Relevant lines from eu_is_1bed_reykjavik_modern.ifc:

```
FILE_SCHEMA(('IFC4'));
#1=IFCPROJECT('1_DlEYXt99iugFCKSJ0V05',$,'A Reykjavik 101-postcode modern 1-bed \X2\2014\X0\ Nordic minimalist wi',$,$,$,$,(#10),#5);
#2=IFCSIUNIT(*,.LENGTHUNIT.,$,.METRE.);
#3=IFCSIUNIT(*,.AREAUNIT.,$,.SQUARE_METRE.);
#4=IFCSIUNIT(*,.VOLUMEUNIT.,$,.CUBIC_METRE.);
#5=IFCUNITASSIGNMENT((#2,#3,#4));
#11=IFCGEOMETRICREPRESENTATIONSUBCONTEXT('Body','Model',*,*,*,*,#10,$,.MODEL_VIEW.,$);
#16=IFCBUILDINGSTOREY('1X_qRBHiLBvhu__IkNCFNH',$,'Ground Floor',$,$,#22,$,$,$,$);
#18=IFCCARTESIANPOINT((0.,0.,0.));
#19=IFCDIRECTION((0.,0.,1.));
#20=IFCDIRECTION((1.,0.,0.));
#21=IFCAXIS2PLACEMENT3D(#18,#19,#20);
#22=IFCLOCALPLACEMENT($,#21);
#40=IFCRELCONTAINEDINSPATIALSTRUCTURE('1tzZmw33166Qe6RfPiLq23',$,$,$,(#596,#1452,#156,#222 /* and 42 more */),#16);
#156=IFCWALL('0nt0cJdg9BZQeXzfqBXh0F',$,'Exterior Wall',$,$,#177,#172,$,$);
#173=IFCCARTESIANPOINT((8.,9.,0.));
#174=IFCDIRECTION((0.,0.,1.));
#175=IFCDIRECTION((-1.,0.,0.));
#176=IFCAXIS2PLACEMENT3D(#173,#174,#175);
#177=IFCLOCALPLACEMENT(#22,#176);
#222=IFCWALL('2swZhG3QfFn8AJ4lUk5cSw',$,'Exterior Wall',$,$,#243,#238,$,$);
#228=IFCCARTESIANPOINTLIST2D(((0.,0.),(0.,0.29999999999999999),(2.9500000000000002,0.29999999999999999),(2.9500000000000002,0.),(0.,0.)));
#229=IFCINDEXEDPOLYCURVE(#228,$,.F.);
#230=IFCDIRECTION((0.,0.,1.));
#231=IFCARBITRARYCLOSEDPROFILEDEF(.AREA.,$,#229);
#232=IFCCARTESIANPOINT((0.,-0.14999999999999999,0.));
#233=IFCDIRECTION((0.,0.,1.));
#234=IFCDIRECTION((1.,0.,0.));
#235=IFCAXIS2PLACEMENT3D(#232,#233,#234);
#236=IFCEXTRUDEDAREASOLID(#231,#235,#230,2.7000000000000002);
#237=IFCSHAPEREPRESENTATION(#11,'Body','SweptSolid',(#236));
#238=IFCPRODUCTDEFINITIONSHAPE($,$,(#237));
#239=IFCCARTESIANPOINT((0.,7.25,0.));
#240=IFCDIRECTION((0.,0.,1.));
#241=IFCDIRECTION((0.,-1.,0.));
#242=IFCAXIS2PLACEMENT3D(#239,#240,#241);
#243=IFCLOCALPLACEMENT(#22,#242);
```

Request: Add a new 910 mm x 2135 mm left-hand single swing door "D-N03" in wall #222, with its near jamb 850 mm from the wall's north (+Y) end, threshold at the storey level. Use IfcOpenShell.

```python
import numpy as np
import ifcopenshell
import ifcopenshell.api.feature
import ifcopenshell.api.geometry
import ifcopenshell.api.root
import ifcopenshell.api.spatial
import ifcopenshell.geom
import ifcopenshell.util.element
import ifcopenshell.util.placement
import ifcopenshell.util.representation
import ifcopenshell.util.shape
import ifcopenshell.util.unit

model = ifcopenshell.open("eu_is_1bed_reykjavik_modern.ifc")
unit_scale = ifcopenshell.util.unit.calculate_unit_scale(model)
settings = ifcopenshell.geom.settings()


def volume(element):
    """Net volume in cubic metres, openings subtracted."""
    shape = ifcopenshell.geom.create_shape(settings, element)
    return ifcopenshell.util.shape.get_volume(shape.geometry)


wall = model.by_guid("2swZhG3QfFn8AJ4lUk5cSw")
storey = ifcopenshell.util.element.get_container(wall, ifc_class="IfcBuildingStorey")
context = ifcopenshell.util.representation.get_context(model, "Model", "Body", "MODEL_VIEW")
before = volume(wall)

width, height, from_end, sill = 0.91, 2.135, 0.85, 0.0  # metres

# The wall runs along its own X axis, and the end named is its -X end.
wall_shape = ifcopenshell.geom.create_shape(settings, wall)
x, y, z = ifcopenshell.util.shape.get_vertices(wall_shape.geometry).T
start = x.min() + from_end
face, thickness = float(y.min()), float(y.max() - y.min())
wall_matrix = ifcopenshell.util.placement.get_local_placement(wall.ObjectPlacement)
level = ifcopenshell.util.placement.get_local_placement(storey.ObjectPlacement)[2, 3]


def in_wall(x, y):
    """Placement at x, y metres in the wall's axes, at sill height."""
    matrix = wall_matrix.copy()
    matrix[:, 3] = wall_matrix @ np.array([x / unit_scale, y / unit_scale, 0.0, 1.0])
    matrix[2, 3] = level + sill / unit_scale
    return matrix


# Opening: a box that overshoots both wall faces by 50 mm.
opening = ifcopenshell.api.root.create_entity(model, ifc_class="IfcOpeningElement", predefined_type="OPENING")
box = ifcopenshell.api.geometry.add_wall_representation(
    model, context=context, length=width, height=height, thickness=thickness + 0.1
)
ifcopenshell.api.geometry.assign_representation(model, product=opening, representation=box)
ifcopenshell.api.geometry.edit_object_placement(model, product=opening, matrix=in_wall(start, face - 0.05), is_si=False)
ifcopenshell.api.feature.add_feature(model, feature=opening, element=wall)

door = ifcopenshell.api.root.create_entity(model, ifc_class="IfcDoor", name="D-N03", predefined_type="DOOR")
door.OverallWidth, door.OverallHeight = width / unit_scale, height / unit_scale
door.OperationType = "SINGLE_SWING_LEFT"
body = ifcopenshell.api.geometry.add_door_representation(
    model,
    context=context,
    overall_width=door.OverallWidth,
    overall_height=door.OverallHeight,
    operation_type="SINGLE_SWING_LEFT",
    lining_properties={"LiningDepth": thickness / unit_scale, "ThresholdDepth": thickness / unit_scale},
)
ifcopenshell.api.geometry.assign_representation(model, product=door, representation=body)
ifcopenshell.api.spatial.assign_container(model, products=[door], relating_structure=storey)
ifcopenshell.api.feature.add_filling(model, opening=opening, element=door)

# The lining spans the wall, so the door starts at the wall face.
ifcopenshell.api.geometry.edit_object_placement(model, product=door, matrix=in_wall(start, face), is_si=False)

after = volume(wall)

print(f"wall volume {before:.3f} -> {after:.3f} m3")

model.write("eu_is_1bed_reykjavik_modern_v2.ifc")
```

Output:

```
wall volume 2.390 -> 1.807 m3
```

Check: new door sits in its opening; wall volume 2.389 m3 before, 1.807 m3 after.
